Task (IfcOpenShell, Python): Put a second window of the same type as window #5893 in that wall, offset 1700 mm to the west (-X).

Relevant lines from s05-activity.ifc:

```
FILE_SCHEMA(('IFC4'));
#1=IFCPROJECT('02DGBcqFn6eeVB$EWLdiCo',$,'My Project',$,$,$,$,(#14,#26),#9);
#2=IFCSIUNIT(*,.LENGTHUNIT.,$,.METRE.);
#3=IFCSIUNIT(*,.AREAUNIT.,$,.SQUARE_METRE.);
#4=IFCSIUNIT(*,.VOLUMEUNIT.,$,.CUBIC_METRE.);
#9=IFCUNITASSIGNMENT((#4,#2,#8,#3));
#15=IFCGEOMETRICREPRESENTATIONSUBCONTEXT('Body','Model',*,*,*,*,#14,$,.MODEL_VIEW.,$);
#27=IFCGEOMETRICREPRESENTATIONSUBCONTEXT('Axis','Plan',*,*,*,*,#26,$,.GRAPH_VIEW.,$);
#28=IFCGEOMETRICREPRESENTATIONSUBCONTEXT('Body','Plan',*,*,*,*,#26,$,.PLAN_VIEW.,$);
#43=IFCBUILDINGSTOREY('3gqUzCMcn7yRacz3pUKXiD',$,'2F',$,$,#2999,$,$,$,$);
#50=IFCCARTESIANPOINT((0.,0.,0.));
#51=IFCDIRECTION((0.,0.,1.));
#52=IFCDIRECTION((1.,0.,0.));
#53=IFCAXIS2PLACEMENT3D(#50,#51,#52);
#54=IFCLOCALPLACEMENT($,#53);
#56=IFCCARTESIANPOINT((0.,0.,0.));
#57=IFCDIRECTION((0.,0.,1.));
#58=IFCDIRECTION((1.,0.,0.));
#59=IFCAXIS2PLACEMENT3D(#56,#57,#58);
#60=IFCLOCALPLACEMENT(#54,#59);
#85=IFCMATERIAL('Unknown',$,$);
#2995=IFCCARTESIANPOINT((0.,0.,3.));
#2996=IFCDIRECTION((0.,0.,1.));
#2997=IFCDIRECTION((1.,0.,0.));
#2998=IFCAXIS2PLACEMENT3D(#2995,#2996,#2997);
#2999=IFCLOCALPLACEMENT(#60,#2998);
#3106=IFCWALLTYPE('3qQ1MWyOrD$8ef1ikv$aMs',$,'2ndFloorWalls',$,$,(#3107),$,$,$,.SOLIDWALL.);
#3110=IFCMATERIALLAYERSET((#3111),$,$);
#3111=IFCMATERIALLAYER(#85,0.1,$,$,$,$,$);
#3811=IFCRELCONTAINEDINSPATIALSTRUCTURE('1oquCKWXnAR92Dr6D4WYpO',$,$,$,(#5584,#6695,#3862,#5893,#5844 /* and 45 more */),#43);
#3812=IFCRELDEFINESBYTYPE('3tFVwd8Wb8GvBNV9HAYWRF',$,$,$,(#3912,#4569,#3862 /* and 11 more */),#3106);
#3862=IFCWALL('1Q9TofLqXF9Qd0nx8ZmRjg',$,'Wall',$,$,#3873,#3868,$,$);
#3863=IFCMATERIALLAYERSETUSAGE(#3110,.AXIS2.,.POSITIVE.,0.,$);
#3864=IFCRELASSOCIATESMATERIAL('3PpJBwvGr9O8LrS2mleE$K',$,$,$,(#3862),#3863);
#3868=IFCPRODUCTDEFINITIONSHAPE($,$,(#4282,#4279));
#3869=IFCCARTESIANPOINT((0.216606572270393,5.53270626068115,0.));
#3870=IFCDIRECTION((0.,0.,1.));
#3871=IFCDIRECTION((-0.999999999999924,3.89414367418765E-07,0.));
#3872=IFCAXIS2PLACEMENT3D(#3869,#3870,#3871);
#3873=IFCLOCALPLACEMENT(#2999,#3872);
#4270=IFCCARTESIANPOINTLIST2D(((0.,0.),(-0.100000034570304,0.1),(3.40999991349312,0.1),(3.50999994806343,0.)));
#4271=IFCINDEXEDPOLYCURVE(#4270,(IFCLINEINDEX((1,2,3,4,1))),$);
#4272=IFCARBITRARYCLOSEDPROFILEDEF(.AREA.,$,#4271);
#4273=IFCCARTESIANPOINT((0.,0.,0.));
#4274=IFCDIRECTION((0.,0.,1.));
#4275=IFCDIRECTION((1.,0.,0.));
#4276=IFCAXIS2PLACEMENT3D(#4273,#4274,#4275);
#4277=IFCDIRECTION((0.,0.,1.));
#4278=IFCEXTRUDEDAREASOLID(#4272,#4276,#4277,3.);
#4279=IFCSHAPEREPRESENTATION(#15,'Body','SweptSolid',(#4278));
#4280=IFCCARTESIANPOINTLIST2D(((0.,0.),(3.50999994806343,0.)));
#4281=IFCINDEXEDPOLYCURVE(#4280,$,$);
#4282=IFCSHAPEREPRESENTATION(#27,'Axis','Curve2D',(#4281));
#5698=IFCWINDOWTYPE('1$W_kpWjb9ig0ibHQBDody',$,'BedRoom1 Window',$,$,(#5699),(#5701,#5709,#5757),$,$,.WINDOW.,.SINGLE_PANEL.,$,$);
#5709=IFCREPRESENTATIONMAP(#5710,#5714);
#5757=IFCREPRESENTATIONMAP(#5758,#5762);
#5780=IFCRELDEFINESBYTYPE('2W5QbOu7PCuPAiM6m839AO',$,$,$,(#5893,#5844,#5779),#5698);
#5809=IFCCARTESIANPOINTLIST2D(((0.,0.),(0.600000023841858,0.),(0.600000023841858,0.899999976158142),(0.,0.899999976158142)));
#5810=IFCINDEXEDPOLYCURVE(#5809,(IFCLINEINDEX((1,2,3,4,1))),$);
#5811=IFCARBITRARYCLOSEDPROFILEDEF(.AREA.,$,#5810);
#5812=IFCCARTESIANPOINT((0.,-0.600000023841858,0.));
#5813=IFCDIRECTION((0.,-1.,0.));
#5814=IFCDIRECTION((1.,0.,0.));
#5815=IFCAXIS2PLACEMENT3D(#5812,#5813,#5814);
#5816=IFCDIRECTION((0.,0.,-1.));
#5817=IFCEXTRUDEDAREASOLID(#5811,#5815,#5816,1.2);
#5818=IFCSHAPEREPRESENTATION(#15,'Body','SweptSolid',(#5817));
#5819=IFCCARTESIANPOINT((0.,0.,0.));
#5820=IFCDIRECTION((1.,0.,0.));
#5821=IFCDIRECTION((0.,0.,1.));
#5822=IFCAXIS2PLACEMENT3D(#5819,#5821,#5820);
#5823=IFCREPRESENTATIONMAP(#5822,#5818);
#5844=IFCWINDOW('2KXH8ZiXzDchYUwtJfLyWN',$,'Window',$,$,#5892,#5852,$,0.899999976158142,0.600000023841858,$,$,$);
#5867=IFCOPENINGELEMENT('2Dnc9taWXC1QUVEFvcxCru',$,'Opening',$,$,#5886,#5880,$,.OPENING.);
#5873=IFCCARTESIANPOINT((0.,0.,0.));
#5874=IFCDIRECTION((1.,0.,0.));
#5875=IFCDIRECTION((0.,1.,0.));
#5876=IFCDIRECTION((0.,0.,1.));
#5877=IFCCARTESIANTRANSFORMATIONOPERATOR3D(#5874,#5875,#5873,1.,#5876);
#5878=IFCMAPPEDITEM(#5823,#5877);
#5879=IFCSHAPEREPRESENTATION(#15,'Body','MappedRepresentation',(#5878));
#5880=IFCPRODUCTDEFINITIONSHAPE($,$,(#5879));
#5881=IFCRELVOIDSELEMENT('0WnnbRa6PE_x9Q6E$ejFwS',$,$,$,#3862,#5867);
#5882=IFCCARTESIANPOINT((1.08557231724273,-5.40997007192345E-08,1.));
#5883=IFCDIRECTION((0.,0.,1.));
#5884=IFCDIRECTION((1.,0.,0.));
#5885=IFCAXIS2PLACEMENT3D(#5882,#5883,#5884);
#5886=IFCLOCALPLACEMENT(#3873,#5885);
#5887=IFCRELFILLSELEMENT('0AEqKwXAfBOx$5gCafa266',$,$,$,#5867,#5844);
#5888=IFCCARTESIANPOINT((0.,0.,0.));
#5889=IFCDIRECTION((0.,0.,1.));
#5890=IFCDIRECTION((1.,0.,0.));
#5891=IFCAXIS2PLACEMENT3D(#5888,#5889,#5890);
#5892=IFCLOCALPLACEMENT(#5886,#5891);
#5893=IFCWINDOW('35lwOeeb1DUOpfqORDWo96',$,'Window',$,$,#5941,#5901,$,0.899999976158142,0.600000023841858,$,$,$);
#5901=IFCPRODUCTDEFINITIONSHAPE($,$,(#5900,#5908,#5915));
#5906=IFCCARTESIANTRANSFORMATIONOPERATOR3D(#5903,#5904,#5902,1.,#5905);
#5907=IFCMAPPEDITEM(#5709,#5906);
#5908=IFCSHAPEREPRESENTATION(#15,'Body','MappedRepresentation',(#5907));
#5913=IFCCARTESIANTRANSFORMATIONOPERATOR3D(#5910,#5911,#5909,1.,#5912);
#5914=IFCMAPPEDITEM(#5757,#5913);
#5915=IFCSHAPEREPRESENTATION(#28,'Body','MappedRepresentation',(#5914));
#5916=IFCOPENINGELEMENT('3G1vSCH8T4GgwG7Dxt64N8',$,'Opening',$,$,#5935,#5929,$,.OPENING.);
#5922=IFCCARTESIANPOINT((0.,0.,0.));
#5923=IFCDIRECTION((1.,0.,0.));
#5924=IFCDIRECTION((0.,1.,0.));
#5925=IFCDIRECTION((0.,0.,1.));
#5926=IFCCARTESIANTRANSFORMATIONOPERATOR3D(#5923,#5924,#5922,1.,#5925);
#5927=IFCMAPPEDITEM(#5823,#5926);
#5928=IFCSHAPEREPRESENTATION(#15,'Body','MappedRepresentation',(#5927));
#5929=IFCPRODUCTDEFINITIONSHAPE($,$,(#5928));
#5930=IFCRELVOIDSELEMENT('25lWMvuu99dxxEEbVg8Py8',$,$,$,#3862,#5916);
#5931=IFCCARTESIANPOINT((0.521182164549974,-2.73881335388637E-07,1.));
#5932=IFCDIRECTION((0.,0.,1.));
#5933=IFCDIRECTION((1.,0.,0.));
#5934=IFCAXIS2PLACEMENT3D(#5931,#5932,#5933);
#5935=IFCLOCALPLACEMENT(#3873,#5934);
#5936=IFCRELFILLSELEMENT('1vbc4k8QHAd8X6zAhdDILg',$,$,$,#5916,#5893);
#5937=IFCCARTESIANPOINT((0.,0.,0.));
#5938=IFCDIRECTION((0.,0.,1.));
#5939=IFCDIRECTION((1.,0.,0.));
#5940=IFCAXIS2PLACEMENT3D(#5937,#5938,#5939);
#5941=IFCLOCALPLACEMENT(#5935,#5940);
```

```python
import ifcopenshell
import ifcopenshell.api.feature
import ifcopenshell.api.geometry
import ifcopenshell.api.root
import ifcopenshell.geom
import ifcopenshell.util.element
import ifcopenshell.util.placement
import ifcopenshell.util.shape
import ifcopenshell.util.unit

model = ifcopenshell.open("s05-activity.ifc")
unit_scale = ifcopenshell.util.unit.calculate_unit_scale(model)
settings = ifcopenshell.geom.settings()


def volume(element):
    """Net volume in cubic metres, openings subtracted."""
    shape = ifcopenshell.geom.create_shape(settings, element)
    return ifcopenshell.util.shape.get_volume(shape.geometry)


window = model.by_id(5893)
opening = window.FillsVoids[0].RelatingOpeningElement
wall = opening.VoidsElements[0].RelatingBuildingElement
before = volume(wall)
shift = ifcopenshell.util.placement.get_local_placement(wall.ObjectPlacement)[:3, 0] * 1.7 / unit_scale

# copy_class copies the void relationship, type, container and properties, but no geometry.
new_opening = ifcopenshell.api.root.copy_class(model, product=opening)
new_opening.Representation = ifcopenshell.util.element.copy_deep(
    model, opening.Representation, exclude=["IfcGeometricRepresentationContext", "IfcRepresentationMap"]
)
new_window = ifcopenshell.api.root.copy_class(model, product=window)
new_window.Representation = ifcopenshell.util.element.copy_deep(
    model, window.Representation, exclude=["IfcGeometricRepresentationContext", "IfcRepresentationMap"]
)
ifcopenshell.api.feature.add_filling(model, opening=new_opening, element=new_window)

for old, new in ((opening, new_opening), (window, new_window)):
    matrix = ifcopenshell.util.placement.get_local_placement(old.ObjectPlacement)
    matrix[:3, 3] += shift
    ifcopenshell.api.geometry.edit_object_placement(model, product=new, matrix=matrix, is_si=False)

after = volume(wall)

print(f"wall volume {before:.3f} -> {after:.3f} m3")

model.write("s05-activity_updated.ifc")
```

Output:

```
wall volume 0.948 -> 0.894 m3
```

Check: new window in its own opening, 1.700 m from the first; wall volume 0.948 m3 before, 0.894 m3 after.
